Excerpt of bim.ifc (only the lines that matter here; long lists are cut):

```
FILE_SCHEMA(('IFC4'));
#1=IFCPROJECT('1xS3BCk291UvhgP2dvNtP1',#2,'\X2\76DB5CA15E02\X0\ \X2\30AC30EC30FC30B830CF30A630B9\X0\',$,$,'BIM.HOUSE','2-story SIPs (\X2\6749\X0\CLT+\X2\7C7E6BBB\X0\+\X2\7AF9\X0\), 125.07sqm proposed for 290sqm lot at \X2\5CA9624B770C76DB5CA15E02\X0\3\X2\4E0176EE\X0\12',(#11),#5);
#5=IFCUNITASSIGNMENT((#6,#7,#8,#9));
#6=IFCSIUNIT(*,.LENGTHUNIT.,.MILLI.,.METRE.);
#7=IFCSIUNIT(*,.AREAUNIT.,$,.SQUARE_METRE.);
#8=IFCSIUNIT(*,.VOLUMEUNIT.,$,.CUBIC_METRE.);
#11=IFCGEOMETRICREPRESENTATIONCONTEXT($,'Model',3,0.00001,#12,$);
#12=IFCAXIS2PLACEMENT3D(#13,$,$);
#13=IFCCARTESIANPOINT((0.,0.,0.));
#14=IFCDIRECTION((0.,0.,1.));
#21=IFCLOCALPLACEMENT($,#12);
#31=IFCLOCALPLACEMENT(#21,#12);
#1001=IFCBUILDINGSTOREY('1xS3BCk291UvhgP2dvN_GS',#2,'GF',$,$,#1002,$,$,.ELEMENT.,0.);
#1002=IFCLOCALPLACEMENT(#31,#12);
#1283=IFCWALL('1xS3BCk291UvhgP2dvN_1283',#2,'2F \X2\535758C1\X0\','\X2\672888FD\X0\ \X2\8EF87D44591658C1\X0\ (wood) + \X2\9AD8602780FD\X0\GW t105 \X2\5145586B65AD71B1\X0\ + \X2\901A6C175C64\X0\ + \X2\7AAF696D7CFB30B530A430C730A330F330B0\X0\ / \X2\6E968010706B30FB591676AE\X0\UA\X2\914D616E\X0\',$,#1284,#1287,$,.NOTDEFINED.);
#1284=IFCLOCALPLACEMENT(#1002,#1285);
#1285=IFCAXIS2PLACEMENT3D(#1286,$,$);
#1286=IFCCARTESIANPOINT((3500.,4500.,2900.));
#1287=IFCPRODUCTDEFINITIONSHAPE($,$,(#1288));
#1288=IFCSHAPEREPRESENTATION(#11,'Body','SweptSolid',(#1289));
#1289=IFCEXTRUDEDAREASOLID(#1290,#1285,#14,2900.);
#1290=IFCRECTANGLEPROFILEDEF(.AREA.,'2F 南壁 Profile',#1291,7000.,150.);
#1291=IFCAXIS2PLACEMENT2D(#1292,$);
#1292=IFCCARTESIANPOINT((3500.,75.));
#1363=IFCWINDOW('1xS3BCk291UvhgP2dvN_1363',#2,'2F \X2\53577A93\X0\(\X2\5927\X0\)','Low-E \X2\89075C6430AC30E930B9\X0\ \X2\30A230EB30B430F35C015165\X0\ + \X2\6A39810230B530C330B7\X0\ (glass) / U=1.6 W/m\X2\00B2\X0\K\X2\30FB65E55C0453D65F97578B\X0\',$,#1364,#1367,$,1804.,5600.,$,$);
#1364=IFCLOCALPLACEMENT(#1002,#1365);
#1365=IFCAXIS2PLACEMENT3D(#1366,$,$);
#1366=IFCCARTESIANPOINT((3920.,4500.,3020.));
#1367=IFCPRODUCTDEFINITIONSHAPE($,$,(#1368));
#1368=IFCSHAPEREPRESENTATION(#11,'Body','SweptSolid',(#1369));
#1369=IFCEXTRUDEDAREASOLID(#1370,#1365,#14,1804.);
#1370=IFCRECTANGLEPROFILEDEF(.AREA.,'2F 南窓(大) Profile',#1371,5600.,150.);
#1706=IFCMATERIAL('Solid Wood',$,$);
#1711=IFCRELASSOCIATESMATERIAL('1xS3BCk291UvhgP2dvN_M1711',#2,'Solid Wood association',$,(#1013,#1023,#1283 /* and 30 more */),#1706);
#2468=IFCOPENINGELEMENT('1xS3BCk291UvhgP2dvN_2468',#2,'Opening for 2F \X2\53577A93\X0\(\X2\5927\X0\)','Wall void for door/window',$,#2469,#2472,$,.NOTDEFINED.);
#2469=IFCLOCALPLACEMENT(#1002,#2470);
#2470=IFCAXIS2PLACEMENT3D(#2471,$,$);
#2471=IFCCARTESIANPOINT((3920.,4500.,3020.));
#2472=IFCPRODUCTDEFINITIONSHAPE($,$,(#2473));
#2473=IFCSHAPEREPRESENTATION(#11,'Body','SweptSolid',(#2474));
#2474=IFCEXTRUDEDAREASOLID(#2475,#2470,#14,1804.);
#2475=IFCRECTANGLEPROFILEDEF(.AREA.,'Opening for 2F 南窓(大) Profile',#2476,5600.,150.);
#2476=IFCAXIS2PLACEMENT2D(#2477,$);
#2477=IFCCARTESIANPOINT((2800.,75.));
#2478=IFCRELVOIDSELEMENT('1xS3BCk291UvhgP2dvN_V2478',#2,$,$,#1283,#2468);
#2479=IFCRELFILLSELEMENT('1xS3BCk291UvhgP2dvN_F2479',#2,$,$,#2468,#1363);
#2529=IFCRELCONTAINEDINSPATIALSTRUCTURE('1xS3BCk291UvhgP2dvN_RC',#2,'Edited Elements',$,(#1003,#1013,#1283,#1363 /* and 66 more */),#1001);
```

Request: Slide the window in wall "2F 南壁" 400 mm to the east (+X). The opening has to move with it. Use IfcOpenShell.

```python
import ifcopenshell
import ifcopenshell.api.geometry
import ifcopenshell.util.placement
import ifcopenshell.util.unit

model = ifcopenshell.open("bim.ifc")
unit_scale = ifcopenshell.util.unit.calculate_unit_scale(model)

window = model.by_guid("1xS3BCk291UvhgP2dvN_1363")
opening = window.FillsVoids[0].RelatingOpeningElement
wall = opening.VoidsElements[0].RelatingBuildingElement

wall_matrix = ifcopenshell.util.placement.get_local_placement(wall.ObjectPlacement)
shift = wall_matrix[:3, 0] * 0.4 / unit_scale
before = ifcopenshell.util.placement.get_local_placement(window.ObjectPlacement)[:3, 3].copy()

# The window is not placed relative to its opening, so move both.
for product in (opening, window):
    matrix = ifcopenshell.util.placement.get_local_placement(product.ObjectPlacement)
    matrix[:3, 3] += shift
    ifcopenshell.api.geometry.edit_object_placement(model, product=product, matrix=matrix, is_si=False)

after = ifcopenshell.util.placement.get_local_placement(window.ObjectPlacement)[:3, 3]
print("window moved by", (after - before).round(3) + 0.0)

model.write("bim_v2.ifc")
```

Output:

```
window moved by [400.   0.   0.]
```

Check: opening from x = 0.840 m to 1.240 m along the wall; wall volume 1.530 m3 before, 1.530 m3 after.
